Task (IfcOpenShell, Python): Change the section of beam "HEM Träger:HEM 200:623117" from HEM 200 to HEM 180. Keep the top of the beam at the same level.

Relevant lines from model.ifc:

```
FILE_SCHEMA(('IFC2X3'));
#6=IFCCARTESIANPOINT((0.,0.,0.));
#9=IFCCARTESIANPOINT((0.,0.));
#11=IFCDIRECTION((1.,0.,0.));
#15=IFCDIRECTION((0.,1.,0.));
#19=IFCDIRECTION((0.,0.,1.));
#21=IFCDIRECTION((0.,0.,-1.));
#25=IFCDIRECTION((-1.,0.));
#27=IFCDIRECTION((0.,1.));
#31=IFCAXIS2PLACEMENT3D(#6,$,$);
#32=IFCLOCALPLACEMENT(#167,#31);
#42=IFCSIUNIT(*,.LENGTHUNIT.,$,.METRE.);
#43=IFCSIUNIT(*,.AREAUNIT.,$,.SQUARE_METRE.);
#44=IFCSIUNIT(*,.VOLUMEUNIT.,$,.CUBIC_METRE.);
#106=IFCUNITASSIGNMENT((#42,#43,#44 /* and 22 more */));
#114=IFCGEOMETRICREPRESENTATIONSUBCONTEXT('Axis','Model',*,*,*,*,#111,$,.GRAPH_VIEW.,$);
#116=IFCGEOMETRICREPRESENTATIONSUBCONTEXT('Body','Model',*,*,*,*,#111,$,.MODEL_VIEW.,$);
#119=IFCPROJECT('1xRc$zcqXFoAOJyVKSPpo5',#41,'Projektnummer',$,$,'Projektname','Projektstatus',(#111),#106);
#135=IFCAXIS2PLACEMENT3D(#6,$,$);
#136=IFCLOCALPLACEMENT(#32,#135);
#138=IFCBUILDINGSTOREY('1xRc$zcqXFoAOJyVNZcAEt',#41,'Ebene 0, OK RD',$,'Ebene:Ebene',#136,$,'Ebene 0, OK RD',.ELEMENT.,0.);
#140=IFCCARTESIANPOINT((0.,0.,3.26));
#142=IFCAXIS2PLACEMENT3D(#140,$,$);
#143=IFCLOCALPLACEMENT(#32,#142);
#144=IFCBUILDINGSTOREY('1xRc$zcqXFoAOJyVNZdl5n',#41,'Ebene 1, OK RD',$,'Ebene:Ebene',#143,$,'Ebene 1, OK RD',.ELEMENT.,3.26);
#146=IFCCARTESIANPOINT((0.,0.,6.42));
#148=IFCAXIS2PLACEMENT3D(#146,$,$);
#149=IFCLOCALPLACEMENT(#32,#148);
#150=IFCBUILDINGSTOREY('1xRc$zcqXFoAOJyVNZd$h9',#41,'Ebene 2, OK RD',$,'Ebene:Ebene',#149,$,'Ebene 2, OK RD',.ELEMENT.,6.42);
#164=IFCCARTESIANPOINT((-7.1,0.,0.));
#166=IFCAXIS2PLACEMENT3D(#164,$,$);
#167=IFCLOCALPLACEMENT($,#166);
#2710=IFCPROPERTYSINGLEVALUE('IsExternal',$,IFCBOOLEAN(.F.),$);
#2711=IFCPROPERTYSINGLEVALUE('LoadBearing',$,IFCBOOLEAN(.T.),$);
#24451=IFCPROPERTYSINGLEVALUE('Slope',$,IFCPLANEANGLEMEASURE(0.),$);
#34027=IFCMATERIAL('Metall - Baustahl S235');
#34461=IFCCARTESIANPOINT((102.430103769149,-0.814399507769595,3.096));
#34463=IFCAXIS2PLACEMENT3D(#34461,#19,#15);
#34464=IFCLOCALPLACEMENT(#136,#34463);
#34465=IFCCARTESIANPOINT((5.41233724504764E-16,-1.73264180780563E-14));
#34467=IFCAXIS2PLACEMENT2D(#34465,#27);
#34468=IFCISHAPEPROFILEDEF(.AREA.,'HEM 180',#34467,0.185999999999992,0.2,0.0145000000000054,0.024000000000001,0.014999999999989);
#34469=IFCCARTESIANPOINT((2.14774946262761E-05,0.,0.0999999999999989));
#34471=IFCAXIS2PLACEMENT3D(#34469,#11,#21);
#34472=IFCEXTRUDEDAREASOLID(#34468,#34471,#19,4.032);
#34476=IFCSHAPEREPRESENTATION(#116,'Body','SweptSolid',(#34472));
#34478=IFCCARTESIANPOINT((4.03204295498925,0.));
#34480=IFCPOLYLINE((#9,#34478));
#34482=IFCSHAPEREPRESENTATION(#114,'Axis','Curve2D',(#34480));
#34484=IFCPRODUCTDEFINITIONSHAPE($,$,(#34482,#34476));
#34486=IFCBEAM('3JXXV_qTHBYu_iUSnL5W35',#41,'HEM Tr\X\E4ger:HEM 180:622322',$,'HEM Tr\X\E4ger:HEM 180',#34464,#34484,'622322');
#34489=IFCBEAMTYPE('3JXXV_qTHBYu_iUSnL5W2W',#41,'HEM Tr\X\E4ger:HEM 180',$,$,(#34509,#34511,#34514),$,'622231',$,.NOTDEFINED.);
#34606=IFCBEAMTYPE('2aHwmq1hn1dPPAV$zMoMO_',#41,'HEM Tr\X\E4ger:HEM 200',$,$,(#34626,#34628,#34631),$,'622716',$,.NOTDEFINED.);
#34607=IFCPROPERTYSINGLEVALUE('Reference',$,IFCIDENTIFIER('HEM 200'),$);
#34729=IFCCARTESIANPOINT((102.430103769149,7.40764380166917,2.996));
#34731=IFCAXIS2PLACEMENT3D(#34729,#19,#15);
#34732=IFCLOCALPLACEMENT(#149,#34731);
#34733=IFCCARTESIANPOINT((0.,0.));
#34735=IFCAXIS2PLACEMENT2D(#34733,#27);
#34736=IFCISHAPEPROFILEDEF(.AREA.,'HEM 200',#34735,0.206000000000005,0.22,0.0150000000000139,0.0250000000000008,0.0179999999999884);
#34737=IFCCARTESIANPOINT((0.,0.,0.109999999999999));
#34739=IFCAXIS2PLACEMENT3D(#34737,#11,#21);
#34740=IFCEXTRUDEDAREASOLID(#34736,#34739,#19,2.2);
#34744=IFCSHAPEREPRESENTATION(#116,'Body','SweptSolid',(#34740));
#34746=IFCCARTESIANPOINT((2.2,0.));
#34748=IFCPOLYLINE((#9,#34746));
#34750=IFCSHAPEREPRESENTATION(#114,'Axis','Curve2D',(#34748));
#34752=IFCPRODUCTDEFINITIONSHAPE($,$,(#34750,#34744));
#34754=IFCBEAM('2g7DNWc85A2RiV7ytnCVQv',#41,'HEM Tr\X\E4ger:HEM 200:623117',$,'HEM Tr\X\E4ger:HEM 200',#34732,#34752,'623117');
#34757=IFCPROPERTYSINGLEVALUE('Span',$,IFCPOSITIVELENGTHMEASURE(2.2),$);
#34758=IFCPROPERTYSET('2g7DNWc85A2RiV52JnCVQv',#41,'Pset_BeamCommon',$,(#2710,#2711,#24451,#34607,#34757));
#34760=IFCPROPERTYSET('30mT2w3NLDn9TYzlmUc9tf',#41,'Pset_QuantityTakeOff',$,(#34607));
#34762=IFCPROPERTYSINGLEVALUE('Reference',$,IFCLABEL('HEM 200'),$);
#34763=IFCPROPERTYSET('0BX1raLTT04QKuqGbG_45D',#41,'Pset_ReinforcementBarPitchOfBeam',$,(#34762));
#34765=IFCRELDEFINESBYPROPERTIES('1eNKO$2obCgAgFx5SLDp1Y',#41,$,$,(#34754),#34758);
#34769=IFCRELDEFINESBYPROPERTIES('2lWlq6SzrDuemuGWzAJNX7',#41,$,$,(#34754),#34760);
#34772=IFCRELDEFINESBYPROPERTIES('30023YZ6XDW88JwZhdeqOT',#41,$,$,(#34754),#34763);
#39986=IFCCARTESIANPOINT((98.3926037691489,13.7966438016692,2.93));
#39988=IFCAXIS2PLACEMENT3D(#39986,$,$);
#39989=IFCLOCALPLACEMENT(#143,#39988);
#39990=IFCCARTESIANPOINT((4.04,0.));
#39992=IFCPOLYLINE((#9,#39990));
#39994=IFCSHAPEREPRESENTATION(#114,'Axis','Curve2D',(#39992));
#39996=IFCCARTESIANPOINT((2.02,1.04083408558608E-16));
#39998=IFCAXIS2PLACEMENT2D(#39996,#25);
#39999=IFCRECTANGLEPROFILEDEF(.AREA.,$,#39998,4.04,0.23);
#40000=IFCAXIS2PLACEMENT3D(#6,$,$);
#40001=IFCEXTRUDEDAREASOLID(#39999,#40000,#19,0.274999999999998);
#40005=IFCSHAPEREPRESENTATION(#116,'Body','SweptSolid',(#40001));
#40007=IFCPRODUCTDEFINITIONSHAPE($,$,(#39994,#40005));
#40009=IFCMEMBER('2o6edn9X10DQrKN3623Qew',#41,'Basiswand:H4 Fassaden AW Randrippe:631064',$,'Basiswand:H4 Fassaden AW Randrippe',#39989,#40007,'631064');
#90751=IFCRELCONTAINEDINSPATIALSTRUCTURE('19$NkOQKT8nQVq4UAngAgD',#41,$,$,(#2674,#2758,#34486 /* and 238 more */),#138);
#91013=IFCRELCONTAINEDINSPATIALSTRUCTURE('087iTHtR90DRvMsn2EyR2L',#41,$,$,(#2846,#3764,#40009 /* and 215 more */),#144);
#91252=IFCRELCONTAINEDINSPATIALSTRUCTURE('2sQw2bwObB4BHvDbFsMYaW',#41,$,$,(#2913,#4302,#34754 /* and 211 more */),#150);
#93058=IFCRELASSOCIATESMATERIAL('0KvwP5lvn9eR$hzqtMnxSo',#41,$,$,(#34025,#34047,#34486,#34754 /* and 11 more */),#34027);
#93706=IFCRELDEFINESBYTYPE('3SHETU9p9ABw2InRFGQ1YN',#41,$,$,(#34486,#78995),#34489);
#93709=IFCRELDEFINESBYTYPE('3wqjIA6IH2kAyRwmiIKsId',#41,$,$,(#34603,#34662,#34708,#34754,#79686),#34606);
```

```python
import ifcopenshell
import ifcopenshell.api.pset
import ifcopenshell.api.type
import ifcopenshell.util.element
import ifcopenshell.util.representation

model = ifcopenshell.open("model.ifc")

member = model.by_guid("2g7DNWc85A2RiV7ytnCVQv")
source = next(p for p in model.by_type("IfcIShapeProfileDef") if p.ProfileName == "HEM 180")

body = ifcopenshell.util.representation.get_representation(member, "Model", "Body")
solid = body.Items[0]
old_profile = solid.SweptArea

# Copy the section's sizes but keep this member's own profile position.
profile = ifcopenshell.util.element.copy(model, source)
# Profiles are centred, so shift by half the change in depth to hold the top.
shift = (old_profile.OverallDepth - profile.OverallDepth) / 2
x, y = old_profile.Position.Location.Coordinates
up = (-1.0, 0.0)  # upwards, in the solid's own plane
location = model.createIfcCartesianPoint((x + up[0] * shift, y + up[1] * shift))
profile.Position = model.createIfcAxis2Placement2D(location, old_profile.Position.RefDirection)
solid.SweptArea = profile
if not model.get_total_inverses(old_profile):
    ifcopenshell.util.element.remove_deep2(model, old_profile)

new_type = model.by_guid("3JXXV_qTHBYu_iUSnL5W2W")
ifcopenshell.api.type.assign_type(
    model, related_objects=[member], relating_type=new_type, should_map_representations=False
)
member.Name = member.Name.replace("HEM 200", "HEM 180")
member.ObjectType = "HEM Träger:HEM 180"
pset = model.by_id(ifcopenshell.util.element.get_pset(member, "Pset_BeamCommon", should_inherit=False)["id"])
ifcopenshell.api.pset.edit_pset(model, pset=pset, properties={"Reference": "HEM 180"})
pset = model.by_id(ifcopenshell.util.element.get_pset(member, "Pset_QuantityTakeOff", should_inherit=False)["id"])
ifcopenshell.api.pset.edit_pset(model, pset=pset, properties={"Reference": "HEM 180"})
pset = model.by_id(ifcopenshell.util.element.get_pset(member, "Pset_ReinforcementBarPitchOfBeam", should_inherit=False)["id"])
ifcopenshell.api.pset.edit_pset(model, pset=pset, properties={"Reference": "HEM 180"})

print(solid.SweptArea)

model.write("model_rev.ifc")
```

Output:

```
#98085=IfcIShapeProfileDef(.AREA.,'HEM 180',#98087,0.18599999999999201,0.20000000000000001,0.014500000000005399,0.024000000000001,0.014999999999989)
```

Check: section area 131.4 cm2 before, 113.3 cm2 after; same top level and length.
